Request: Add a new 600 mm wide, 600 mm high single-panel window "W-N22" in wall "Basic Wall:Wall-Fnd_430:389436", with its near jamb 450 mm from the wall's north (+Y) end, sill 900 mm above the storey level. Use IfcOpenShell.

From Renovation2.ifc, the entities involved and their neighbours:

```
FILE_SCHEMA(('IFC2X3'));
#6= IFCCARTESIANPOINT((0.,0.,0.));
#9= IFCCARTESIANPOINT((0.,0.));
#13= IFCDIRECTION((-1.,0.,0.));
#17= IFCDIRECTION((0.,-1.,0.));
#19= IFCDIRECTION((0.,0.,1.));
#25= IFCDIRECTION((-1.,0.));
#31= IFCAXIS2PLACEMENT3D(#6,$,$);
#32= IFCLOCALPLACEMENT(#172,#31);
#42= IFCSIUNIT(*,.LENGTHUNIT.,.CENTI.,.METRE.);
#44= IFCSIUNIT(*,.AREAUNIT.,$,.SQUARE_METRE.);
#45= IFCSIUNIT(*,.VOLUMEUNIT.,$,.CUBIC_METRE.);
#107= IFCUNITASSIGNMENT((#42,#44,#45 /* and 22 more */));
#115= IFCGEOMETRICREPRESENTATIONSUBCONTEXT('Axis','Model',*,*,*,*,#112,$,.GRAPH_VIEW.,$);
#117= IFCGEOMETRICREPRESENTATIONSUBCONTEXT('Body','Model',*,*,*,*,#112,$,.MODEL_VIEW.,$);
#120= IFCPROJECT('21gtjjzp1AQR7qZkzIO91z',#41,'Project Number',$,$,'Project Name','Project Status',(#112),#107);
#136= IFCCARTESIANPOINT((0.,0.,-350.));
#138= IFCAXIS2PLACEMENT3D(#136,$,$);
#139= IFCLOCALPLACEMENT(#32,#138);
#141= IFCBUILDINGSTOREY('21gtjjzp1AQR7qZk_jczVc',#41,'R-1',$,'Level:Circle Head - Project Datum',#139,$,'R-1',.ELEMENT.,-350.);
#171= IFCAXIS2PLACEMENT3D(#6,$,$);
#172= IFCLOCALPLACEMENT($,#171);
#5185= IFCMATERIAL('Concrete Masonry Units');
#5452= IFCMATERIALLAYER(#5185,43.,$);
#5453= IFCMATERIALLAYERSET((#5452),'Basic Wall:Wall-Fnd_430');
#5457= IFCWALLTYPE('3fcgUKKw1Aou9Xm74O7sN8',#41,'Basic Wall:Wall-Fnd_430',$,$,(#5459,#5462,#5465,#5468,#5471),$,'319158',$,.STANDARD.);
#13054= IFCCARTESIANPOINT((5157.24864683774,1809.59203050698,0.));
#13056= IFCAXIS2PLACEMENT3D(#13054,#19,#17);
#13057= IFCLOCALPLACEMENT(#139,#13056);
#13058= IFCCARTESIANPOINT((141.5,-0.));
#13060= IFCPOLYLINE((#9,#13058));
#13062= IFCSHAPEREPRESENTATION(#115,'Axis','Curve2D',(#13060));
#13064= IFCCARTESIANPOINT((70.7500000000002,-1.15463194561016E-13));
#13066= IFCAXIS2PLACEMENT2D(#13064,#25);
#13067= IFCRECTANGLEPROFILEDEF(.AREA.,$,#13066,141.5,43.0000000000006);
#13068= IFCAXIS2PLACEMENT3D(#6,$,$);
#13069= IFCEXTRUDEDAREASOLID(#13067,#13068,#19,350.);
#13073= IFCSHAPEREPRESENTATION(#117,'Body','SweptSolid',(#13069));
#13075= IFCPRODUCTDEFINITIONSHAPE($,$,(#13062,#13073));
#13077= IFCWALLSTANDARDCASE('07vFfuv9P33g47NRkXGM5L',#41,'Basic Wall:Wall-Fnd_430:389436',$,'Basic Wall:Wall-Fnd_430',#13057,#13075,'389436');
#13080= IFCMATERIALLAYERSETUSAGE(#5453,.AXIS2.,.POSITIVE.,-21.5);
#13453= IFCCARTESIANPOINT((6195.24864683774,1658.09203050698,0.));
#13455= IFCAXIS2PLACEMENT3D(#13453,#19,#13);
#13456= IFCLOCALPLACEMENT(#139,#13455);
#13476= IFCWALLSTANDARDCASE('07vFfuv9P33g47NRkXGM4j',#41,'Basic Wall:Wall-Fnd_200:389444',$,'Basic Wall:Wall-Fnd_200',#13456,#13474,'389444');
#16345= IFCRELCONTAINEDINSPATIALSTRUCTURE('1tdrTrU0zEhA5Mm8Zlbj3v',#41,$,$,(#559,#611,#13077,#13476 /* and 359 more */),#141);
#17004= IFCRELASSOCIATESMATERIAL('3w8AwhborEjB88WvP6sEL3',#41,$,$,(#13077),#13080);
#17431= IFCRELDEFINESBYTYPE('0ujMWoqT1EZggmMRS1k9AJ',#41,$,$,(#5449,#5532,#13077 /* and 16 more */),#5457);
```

```python
import numpy as np
import ifcopenshell
import ifcopenshell.api.feature
import ifcopenshell.api.geometry
import ifcopenshell.api.root
import ifcopenshell.api.spatial
import ifcopenshell.api.type
import ifcopenshell.geom
import ifcopenshell.util.element
import ifcopenshell.util.placement
import ifcopenshell.util.representation
import ifcopenshell.util.shape
import ifcopenshell.util.unit

model = ifcopenshell.open("Renovation2.ifc")
unit_scale = ifcopenshell.util.unit.calculate_unit_scale(model)
settings = ifcopenshell.geom.settings()


def volume(element):
    """Net volume in cubic metres, openings subtracted."""
    shape = ifcopenshell.geom.create_shape(settings, element)
    return ifcopenshell.util.shape.get_volume(shape.geometry)


wall = model.by_id(13077)
storey = ifcopenshell.util.element.get_container(wall, ifc_class="IfcBuildingStorey")
context = ifcopenshell.util.representation.get_context(model, "Model", "Body", "MODEL_VIEW")
before = volume(wall)

width, height, from_end, sill = 0.6, 0.6, 0.45, 0.9  # metres

# The wall runs along its own X axis, and the end named is its -X end.
wall_shape = ifcopenshell.geom.create_shape(settings, wall)
x, y, z = ifcopenshell.util.shape.get_vertices(wall_shape.geometry).T
start = x.min() + from_end
face, thickness = float(y.min()), float(y.max() - y.min())
wall_matrix = ifcopenshell.util.placement.get_local_placement(wall.ObjectPlacement)
level = ifcopenshell.util.placement.get_local_placement(storey.ObjectPlacement)[2, 3]


def in_wall(x, y):
    """Placement at x, y metres in the wall's axes, at sill height."""
    matrix = wall_matrix.copy()
    matrix[:, 3] = wall_matrix @ np.array([x / unit_scale, y / unit_scale, 0.0, 1.0])
    matrix[2, 3] = level + sill / unit_scale
    return matrix


# Opening: a box that overshoots both wall faces by 50 mm.
opening = ifcopenshell.api.root.create_entity(model, ifc_class="IfcOpeningElement")
box = ifcopenshell.api.geometry.add_wall_representation(
    model, context=context, length=width, height=height, thickness=thickness + 0.1
)
ifcopenshell.api.geometry.assign_representation(model, product=opening, representation=box)
ifcopenshell.api.geometry.edit_object_placement(model, product=opening, matrix=in_wall(start, face - 0.05), is_si=False)
ifcopenshell.api.feature.add_feature(model, feature=opening, element=wall)

window = ifcopenshell.api.root.create_entity(model, ifc_class="IfcWindow", name="W-N22")
window.OverallWidth, window.OverallHeight = width / unit_scale, height / unit_scale
body = ifcopenshell.api.geometry.add_window_representation(
    model,
    context=context,
    overall_width=window.OverallWidth,
    overall_height=window.OverallHeight,
    partition_type="SINGLE_PANEL",
)
ifcopenshell.api.geometry.assign_representation(model, product=window, representation=body)
ifcopenshell.api.spatial.assign_container(model, products=[window], relating_structure=storey)
fills = ifcopenshell.api.feature.add_filling(model, opening=opening, element=window)
fills.OwnerHistory = window.OwnerHistory  # required in IFC2X3

# IFC2X3 keeps the operation on the window style.
style = ifcopenshell.api.root.create_entity(model, ifc_class="IfcWindowStyle", name="W-N22")
style.OperationType, style.ConstructionType = "SINGLE_PANEL", "NOTDEFINED"
style.ParameterTakesPrecedence = style.Sizeable = False
ifcopenshell.api.type.assign_type(model, related_objects=[window], relating_type=style)

# Centre the window in the wall's thickness.
ifcopenshell.api.geometry.edit_object_placement(model, product=window, matrix=in_wall(start, face), is_si=False)
window_shape = ifcopenshell.geom.create_shape(settings, window)
depth = ifcopenshell.util.shape.get_vertices(window_shape.geometry)[:, 1]
offset = face + thickness / 2 - (depth.min() + depth.max()) / 2
ifcopenshell.api.geometry.edit_object_placement(model, product=window, matrix=in_wall(start, offset), is_si=False)

after = volume(wall)

print(f"wall volume {before:.3f} -> {after:.3f} m3")

model.write("Renovation2-out.ifc")
```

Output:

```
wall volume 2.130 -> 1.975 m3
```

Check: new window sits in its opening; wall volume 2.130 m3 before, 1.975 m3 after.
